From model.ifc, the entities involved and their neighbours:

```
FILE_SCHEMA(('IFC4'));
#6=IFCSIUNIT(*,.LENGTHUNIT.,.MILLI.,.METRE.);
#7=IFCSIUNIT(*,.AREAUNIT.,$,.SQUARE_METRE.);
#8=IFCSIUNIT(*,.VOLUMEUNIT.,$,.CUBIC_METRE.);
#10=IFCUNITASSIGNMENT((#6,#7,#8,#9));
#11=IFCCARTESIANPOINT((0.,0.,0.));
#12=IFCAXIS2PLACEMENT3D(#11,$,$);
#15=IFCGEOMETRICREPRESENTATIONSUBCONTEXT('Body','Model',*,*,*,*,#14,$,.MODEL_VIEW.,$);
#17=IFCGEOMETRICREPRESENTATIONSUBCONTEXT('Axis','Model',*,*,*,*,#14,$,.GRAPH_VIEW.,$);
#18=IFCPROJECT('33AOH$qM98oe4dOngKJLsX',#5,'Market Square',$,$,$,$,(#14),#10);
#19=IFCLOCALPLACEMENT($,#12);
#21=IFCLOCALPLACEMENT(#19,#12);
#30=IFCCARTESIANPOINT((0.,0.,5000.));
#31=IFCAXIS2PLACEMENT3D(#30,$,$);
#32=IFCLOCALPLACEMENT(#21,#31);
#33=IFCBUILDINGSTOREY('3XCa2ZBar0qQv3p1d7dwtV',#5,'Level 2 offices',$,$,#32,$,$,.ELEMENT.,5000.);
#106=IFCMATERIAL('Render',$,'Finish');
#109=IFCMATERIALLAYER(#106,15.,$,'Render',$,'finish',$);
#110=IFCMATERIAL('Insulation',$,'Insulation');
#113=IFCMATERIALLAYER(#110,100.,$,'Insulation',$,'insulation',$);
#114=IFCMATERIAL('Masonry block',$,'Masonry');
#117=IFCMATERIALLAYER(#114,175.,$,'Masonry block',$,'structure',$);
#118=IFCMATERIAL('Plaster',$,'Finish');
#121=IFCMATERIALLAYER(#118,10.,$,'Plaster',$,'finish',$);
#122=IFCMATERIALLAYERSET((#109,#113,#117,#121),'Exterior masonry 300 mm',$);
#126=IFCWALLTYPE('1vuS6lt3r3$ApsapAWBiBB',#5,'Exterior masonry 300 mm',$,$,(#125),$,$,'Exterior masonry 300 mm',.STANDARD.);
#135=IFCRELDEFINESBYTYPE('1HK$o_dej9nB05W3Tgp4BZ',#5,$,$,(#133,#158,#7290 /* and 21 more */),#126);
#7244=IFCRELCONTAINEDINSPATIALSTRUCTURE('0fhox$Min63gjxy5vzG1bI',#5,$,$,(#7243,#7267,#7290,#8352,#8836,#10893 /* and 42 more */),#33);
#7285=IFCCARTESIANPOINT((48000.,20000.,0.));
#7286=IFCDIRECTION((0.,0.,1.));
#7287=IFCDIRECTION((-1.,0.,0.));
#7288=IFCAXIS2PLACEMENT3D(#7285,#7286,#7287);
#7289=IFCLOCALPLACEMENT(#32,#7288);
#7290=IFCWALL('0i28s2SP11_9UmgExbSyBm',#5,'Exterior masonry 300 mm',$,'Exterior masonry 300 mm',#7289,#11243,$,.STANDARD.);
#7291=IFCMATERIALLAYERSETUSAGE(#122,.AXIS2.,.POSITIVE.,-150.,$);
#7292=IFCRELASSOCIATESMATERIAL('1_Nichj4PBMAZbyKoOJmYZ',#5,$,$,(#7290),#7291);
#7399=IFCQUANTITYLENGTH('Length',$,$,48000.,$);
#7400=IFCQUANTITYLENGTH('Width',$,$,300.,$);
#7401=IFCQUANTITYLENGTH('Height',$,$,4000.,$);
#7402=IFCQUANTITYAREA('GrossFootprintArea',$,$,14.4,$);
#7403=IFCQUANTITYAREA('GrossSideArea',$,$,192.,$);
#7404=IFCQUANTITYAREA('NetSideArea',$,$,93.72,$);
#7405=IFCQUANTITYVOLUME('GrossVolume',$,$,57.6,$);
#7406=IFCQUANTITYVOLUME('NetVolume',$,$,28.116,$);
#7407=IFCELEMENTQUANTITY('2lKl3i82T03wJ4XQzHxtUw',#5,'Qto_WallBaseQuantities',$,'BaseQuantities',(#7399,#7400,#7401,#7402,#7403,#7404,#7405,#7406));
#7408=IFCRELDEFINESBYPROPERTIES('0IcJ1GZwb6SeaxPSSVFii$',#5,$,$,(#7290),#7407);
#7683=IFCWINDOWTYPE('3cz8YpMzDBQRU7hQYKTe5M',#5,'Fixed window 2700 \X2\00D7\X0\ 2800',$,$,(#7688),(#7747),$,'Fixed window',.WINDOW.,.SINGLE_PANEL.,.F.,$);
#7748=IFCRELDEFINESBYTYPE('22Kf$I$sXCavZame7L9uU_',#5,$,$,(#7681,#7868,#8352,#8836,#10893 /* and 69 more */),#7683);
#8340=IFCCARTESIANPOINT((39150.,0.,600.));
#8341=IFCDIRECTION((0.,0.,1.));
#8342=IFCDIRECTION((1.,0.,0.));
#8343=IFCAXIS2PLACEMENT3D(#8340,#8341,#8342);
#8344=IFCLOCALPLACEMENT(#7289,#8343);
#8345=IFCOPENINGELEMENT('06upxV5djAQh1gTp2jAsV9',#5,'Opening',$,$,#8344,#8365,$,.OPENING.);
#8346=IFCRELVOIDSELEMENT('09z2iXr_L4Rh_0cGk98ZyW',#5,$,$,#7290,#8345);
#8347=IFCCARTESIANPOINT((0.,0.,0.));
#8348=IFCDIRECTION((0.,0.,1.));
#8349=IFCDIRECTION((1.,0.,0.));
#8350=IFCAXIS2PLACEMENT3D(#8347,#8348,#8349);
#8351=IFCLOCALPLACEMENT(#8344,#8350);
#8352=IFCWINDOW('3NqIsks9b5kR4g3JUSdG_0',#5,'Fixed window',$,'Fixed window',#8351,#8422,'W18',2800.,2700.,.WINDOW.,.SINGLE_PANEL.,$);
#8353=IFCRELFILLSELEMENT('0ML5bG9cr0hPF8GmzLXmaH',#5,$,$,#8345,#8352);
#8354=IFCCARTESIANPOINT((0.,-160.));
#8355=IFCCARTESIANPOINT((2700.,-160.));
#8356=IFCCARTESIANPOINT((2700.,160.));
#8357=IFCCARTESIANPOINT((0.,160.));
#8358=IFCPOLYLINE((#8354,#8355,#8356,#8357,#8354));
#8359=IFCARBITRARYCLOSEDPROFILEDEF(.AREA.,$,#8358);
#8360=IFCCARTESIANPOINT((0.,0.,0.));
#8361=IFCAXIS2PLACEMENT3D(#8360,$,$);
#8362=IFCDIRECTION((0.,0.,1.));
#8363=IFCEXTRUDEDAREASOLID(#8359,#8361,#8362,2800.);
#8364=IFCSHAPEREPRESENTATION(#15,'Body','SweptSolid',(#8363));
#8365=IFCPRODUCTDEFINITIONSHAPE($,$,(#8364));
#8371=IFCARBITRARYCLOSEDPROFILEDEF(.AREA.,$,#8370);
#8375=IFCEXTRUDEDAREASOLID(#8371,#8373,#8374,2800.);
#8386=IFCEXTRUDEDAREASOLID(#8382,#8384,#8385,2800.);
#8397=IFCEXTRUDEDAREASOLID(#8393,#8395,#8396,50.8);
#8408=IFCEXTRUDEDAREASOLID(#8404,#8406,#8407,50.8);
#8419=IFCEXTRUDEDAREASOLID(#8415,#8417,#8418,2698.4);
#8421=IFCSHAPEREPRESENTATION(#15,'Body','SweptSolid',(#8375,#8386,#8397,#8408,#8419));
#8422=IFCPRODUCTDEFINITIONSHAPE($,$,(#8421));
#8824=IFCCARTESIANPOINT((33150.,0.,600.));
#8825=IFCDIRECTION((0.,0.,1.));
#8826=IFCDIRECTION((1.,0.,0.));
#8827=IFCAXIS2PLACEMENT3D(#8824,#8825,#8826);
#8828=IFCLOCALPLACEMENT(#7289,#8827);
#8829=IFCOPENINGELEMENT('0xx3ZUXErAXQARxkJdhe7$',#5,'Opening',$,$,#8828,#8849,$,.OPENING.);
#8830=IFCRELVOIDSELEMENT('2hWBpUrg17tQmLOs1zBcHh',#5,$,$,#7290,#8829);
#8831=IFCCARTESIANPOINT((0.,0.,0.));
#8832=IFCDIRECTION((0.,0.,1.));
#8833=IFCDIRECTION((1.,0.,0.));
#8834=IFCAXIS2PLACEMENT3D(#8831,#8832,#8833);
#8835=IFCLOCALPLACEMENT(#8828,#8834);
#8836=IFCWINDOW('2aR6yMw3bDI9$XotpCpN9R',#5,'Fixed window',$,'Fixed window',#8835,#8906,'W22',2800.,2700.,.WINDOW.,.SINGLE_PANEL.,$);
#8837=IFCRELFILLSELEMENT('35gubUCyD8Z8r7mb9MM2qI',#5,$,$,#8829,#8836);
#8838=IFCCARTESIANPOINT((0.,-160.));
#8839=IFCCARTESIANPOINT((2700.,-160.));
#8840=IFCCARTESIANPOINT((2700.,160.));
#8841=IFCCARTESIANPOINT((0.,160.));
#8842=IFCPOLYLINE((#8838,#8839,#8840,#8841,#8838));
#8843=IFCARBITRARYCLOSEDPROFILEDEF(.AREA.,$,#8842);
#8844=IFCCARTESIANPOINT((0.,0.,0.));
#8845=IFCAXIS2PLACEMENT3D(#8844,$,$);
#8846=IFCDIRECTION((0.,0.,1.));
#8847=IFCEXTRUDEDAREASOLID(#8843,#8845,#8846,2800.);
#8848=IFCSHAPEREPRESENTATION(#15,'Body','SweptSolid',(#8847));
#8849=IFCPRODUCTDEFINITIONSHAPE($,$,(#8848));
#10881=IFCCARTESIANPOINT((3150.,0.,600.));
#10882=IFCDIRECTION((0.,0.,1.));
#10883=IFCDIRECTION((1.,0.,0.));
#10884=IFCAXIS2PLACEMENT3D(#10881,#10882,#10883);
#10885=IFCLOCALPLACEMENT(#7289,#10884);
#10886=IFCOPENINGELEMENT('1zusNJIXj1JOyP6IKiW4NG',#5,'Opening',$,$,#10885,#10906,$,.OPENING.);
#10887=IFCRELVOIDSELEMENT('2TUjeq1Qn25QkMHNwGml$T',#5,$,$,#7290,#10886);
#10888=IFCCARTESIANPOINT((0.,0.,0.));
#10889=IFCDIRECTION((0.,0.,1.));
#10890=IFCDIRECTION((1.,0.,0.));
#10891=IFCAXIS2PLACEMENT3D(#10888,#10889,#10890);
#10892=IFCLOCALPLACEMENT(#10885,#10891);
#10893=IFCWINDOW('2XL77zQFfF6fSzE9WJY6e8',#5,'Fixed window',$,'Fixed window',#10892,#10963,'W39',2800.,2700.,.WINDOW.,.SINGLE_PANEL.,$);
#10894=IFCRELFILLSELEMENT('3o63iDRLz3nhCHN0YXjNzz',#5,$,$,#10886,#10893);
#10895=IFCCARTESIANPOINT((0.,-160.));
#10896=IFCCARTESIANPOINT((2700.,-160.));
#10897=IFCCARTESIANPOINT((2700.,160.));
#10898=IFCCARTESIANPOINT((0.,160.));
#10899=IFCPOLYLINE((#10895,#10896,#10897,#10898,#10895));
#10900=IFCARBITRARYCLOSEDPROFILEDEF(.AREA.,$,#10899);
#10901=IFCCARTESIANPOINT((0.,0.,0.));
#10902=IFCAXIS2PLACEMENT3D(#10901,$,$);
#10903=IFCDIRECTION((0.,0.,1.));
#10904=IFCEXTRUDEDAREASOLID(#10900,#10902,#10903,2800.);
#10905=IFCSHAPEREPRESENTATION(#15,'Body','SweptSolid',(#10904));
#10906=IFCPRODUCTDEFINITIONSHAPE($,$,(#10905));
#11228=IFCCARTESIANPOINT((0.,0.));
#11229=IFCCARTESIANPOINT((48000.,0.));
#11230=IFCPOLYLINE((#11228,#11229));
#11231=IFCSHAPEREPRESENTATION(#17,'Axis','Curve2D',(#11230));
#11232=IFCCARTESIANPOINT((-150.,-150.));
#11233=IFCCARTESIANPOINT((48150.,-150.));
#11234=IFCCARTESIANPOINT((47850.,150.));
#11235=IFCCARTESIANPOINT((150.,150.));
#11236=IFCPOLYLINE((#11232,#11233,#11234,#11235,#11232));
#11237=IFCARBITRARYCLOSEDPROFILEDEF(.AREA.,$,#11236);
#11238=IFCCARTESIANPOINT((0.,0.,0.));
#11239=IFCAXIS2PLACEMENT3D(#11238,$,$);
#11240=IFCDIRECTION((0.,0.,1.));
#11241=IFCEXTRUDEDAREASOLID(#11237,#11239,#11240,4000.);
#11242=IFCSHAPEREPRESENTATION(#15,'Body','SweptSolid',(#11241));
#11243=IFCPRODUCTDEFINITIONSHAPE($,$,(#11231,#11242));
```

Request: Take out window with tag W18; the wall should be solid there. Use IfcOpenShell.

```python
import ifcopenshell
import ifcopenshell.api.feature
import ifcopenshell.api.pset
import ifcopenshell.api.root
import ifcopenshell.geom
import ifcopenshell.util.element
import ifcopenshell.util.shape
import ifcopenshell.util.unit

model = ifcopenshell.open("model.ifc")
area_scale = ifcopenshell.util.unit.calculate_unit_scale(model, "AREAUNIT")
volume_scale = ifcopenshell.util.unit.calculate_unit_scale(model, "VOLUMEUNIT")
settings = ifcopenshell.geom.settings()


def volume(element):
    """Net volume in cubic metres, openings subtracted."""
    shape = ifcopenshell.geom.create_shape(settings, element)
    return ifcopenshell.util.shape.get_volume(shape.geometry)


window = model.by_guid("3NqIsks9b5kR4g3JUSdG_0")
opening = window.FillsVoids[0].RelatingOpeningElement
wall = opening.VoidsElements[0].RelatingBuildingElement
before = volume(wall)

ifcopenshell.api.root.remove_product(model, product=window)
ifcopenshell.api.feature.remove_feature(model, feature=opening)

after = volume(wall)
thickness = 0.3  # wall thickness in metres

# Update the wall's stored quantities.
qto = model.by_id(ifcopenshell.util.element.get_pset(wall, "Qto_WallBaseQuantities", should_inherit=False)["id"])
ifcopenshell.api.pset.edit_qto(model, qto=qto, properties={
    "NetSideArea": after / thickness / area_scale,
    "NetVolume": after / volume_scale,
})

print(f"wall volume {before:.3f} -> {after:.3f} m3")

model.write("model_v2.ifc")
```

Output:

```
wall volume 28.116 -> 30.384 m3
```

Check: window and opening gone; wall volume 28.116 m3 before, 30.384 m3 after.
